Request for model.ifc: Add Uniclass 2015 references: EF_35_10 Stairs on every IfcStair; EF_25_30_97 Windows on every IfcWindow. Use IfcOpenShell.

First a look at what the model holds.

```python
import ifcopenshell

model = ifcopenshell.open("model.ifc")
print(model.schema)
print("classifications:", [c.Name for c in model.by_type("IfcClassification")])
for ifc_class in ("IfcDoor", "IfcRoof", "IfcStair", "IfcWall", "IfcWindow"):
    print(ifc_class, len(model.by_type(ifc_class)))
```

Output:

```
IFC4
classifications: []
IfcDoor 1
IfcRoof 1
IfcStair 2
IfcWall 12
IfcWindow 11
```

```python
import ifcopenshell
import ifcopenshell.api.classification

model = ifcopenshell.open("model.ifc")

system = ifcopenshell.api.classification.add_classification(model, classification="Uniclass 2015")

codes = {
    "IfcStair": ("EF_35_10", "Stairs"),
    "IfcWindow": ("EF_25_30_97", "Windows"),
}
for ifc_class, (code, name) in codes.items():
    products = model.by_type(ifc_class)
    ifcopenshell.api.classification.add_reference(
        model, products=products, classification=system, identification=code, name=name
    )
    print(code, len(products))

model.write("model_edited.ifc")
```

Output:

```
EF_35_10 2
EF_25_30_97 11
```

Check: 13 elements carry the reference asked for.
